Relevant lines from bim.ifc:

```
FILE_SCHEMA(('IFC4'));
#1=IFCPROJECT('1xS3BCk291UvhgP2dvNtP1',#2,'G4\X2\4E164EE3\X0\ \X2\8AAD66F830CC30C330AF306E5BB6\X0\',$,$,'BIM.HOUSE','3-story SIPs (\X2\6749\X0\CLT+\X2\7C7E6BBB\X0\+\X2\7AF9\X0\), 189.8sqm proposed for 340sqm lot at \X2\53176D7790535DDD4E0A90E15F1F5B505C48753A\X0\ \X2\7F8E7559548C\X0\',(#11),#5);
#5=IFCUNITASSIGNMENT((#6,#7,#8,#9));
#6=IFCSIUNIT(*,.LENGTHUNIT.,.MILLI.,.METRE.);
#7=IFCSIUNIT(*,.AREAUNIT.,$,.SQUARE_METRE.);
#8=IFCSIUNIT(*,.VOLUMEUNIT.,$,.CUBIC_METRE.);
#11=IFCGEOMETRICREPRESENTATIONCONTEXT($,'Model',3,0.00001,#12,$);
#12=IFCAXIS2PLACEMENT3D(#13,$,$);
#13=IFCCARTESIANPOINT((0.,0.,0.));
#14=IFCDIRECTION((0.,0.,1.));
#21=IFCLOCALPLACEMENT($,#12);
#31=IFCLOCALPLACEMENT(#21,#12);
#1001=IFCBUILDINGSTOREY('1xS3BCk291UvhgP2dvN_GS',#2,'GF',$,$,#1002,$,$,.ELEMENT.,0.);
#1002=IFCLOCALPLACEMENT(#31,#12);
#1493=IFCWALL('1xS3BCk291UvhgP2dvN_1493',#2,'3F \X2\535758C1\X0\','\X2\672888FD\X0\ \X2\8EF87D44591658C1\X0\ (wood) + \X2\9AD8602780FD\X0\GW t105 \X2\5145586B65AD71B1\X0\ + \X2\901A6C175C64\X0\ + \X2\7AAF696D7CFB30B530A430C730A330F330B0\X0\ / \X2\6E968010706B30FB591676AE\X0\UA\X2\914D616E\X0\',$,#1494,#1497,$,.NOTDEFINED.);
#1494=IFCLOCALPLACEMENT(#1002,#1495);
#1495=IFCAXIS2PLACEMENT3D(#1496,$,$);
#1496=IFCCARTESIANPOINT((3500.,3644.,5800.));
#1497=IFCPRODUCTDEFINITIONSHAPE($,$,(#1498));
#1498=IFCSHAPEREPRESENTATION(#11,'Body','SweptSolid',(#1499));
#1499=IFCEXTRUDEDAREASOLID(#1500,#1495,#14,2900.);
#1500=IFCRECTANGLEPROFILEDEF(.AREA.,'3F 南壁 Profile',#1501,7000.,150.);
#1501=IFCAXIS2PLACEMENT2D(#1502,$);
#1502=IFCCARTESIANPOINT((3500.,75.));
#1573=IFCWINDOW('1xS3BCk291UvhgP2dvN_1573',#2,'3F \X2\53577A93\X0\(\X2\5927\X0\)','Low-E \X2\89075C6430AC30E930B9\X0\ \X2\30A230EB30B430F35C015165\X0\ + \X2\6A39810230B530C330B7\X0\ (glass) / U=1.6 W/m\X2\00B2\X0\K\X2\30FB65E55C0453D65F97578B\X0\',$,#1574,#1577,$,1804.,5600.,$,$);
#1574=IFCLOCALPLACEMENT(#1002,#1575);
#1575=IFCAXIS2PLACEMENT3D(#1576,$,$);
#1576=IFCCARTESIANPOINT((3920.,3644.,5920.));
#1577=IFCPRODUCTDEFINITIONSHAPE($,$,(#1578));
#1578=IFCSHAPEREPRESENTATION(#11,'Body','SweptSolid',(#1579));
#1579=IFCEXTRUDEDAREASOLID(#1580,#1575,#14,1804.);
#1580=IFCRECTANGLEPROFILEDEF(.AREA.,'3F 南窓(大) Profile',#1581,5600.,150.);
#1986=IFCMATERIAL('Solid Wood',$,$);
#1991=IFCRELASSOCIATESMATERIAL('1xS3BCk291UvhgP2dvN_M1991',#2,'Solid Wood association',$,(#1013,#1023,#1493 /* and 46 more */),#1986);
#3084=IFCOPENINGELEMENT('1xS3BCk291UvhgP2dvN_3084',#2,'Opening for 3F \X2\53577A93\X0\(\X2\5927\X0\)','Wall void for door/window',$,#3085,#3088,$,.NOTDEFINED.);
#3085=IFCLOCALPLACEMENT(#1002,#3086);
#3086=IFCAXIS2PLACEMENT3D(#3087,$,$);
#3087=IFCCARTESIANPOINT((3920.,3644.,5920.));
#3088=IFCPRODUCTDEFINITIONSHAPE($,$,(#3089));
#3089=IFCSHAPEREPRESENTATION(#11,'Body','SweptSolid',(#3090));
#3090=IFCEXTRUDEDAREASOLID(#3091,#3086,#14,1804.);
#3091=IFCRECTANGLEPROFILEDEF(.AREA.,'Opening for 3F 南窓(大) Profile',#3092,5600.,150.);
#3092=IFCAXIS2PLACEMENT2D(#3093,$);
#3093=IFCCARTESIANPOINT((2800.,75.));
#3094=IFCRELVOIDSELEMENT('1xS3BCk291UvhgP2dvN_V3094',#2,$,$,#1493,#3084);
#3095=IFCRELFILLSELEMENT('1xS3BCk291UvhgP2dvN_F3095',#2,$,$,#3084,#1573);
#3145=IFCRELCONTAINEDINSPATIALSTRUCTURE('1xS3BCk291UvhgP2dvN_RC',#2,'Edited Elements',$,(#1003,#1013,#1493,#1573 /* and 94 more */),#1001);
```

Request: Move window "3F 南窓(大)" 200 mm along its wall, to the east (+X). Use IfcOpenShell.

```python
import ifcopenshell
import ifcopenshell.api.geometry
import ifcopenshell.util.placement

model = ifcopenshell.open("bim.ifc")

window = model.by_guid("1xS3BCk291UvhgP2dvN_1573")
opening = window.FillsVoids[0].RelatingOpeningElement
wall = opening.VoidsElements[0].RelatingBuildingElement

wall_matrix = ifcopenshell.util.placement.get_local_placement(wall.ObjectPlacement)
shift = wall_matrix[:3, 0] * 200.0
before = ifcopenshell.util.placement.get_local_placement(window.ObjectPlacement)[:3, 3].copy()

# The window is not placed relative to its opening, so move both.
for product in (opening, window):
    matrix = ifcopenshell.util.placement.get_local_placement(product.ObjectPlacement)
    matrix[:3, 3] += shift
    ifcopenshell.api.geometry.edit_object_placement(model, product=product, matrix=matrix, is_si=False)

after = ifcopenshell.util.placement.get_local_placement(window.ObjectPlacement)[:3, 3]
print("window moved by", (after - before).round(3) + 0.0)

model.write("bim_v2.ifc")
```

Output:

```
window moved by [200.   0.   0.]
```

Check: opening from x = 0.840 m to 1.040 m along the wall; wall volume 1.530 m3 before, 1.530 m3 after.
